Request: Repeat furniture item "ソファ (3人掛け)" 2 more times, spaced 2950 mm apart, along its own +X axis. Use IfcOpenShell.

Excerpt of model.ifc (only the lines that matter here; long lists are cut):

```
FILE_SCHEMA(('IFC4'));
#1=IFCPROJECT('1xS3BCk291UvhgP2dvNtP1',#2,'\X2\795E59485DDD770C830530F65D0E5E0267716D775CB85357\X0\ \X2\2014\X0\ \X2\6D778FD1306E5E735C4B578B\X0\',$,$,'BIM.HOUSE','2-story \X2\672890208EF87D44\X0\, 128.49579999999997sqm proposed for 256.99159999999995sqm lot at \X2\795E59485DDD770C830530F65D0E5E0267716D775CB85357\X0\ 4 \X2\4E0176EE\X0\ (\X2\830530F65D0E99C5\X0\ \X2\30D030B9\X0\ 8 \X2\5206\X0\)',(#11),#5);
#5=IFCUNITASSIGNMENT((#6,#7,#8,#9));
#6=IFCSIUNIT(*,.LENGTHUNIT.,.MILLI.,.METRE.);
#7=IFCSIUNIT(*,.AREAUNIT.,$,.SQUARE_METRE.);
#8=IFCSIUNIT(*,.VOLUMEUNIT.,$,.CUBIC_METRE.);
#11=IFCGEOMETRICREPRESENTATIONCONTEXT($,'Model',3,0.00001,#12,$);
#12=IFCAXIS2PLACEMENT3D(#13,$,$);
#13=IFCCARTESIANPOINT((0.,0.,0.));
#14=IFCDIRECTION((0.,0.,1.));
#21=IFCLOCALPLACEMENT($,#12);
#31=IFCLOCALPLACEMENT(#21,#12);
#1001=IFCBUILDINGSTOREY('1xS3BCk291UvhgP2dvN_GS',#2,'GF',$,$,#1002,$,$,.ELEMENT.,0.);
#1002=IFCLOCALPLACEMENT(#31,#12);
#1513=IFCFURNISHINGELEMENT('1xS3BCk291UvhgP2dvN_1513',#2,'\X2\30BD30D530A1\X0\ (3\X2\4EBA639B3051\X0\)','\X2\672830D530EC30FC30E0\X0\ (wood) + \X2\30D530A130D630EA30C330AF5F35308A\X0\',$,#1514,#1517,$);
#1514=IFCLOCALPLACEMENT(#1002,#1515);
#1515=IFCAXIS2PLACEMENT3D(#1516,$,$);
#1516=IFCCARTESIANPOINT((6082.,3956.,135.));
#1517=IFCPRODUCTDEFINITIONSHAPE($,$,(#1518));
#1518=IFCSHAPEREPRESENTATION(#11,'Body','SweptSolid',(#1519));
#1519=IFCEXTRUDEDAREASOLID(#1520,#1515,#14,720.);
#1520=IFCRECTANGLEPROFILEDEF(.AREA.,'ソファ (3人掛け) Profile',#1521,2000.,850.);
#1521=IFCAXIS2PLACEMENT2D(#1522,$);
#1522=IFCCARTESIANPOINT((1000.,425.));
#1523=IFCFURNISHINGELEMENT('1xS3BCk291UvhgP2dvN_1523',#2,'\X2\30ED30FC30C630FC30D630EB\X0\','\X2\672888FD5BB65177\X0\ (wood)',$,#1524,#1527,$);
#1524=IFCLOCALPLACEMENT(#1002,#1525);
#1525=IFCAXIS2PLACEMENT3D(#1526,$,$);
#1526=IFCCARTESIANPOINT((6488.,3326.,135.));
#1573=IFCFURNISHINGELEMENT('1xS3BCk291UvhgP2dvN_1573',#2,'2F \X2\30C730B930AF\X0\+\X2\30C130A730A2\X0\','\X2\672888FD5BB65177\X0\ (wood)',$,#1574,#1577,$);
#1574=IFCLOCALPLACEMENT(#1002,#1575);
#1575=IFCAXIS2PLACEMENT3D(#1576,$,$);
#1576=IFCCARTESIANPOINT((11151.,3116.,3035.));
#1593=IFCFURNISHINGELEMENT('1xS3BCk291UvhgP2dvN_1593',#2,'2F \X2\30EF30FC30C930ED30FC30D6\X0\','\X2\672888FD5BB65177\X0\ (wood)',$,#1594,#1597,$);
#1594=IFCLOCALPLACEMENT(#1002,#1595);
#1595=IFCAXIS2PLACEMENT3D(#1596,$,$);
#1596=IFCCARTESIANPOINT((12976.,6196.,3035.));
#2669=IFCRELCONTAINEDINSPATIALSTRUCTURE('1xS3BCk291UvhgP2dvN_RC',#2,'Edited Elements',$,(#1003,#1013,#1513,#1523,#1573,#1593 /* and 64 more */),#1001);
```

```python
import ifcopenshell
import ifcopenshell.api.geometry
import ifcopenshell.api.root
import ifcopenshell.util.element
import ifcopenshell.util.placement
import ifcopenshell.util.unit

model = ifcopenshell.open("model.ifc")
unit_scale = ifcopenshell.util.unit.calculate_unit_scale(model)


def reuse_history(source, copy):
    """copy_class also copies each property set's owner history, people and application; keep the originals."""
    for rel in copy.IsDefinedBy:
        if rel.is_a("IfcRelDefinesByProperties") and (history := rel.RelatingPropertyDefinition.OwnerHistory):
            rel.RelatingPropertyDefinition.OwnerHistory = source.OwnerHistory
            ifcopenshell.util.element.remove_deep2(model, history)


source = model.by_id(1513)
base = ifcopenshell.util.placement.get_local_placement(source.ObjectPlacement)
step = base[:3, 0] * 2.95 / unit_scale

for i in range(1, 3):
    copy = ifcopenshell.api.root.copy_class(model, product=source)
    copy.Representation = ifcopenshell.util.element.copy_deep(
        model, source.Representation, exclude=["IfcGeometricRepresentationContext", "IfcRepresentationMap"]
    )
    reuse_history(source, copy)
    matrix = base.copy()
    matrix[:3, 3] += i * step
    print("added at", matrix[:3, 3].round(3) + 0.0)
    ifcopenshell.api.geometry.edit_object_placement(model, product=copy, matrix=matrix, is_si=False)

model.write("model_updated.ifc")
```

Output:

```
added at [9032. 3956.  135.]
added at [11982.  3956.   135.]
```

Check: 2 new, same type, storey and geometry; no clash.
